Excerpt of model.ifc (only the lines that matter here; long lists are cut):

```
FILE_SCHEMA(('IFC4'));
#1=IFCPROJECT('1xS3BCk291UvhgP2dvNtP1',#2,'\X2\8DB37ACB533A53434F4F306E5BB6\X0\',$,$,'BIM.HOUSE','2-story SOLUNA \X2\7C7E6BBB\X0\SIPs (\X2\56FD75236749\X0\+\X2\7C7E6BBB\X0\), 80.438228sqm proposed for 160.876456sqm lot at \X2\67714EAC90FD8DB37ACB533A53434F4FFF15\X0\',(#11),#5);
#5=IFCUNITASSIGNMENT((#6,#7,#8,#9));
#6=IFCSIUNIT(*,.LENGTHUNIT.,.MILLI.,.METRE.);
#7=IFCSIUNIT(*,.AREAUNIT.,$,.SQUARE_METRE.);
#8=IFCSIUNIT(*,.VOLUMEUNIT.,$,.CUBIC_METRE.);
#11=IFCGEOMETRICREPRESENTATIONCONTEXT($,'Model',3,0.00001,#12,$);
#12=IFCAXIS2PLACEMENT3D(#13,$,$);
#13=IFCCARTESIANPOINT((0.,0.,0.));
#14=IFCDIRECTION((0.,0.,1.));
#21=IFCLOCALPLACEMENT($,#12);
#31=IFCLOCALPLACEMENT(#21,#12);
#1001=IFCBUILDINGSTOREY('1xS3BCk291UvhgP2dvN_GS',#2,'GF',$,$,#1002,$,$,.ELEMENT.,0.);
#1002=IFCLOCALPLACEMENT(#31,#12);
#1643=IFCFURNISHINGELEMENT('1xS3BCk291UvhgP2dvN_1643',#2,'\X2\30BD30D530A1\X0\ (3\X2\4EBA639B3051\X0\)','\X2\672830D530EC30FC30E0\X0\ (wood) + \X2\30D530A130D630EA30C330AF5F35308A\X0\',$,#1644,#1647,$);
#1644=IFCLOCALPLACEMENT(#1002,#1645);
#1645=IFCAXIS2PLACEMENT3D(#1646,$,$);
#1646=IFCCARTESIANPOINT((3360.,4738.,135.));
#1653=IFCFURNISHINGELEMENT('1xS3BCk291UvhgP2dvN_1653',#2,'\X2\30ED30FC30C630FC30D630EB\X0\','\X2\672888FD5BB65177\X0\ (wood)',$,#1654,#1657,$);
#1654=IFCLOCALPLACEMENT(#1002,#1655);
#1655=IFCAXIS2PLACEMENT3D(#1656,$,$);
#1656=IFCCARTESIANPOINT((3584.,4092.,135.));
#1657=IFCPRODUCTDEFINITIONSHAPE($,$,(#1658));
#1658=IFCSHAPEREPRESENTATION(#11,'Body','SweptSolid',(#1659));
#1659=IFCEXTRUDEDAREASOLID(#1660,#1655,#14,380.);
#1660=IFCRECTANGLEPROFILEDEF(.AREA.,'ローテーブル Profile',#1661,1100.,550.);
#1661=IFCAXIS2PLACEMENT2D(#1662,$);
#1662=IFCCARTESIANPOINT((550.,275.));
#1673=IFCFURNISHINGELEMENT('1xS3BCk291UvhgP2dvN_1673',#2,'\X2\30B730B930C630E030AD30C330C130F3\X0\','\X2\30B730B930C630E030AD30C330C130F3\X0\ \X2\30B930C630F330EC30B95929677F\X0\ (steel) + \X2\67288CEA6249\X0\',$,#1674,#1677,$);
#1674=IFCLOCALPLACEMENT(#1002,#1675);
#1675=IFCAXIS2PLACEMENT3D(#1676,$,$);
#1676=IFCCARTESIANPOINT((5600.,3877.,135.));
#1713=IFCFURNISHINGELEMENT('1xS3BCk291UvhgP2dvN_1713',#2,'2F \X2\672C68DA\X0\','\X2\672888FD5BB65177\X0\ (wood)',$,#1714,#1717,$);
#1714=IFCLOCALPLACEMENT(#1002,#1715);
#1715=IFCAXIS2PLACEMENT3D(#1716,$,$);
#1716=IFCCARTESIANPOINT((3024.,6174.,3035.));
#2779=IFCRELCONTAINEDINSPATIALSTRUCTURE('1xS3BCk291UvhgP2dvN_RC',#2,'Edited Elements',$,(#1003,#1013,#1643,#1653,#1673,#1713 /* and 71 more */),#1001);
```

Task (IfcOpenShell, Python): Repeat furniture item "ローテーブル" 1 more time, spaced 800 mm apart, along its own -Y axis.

```python
import ifcopenshell
import ifcopenshell.api.geometry
import ifcopenshell.api.root
import ifcopenshell.util.element
import ifcopenshell.util.placement
import ifcopenshell.util.unit

model = ifcopenshell.open("model.ifc")
unit_scale = ifcopenshell.util.unit.calculate_unit_scale(model)


def reuse_history(source, copy):
    """copy_class also copies each property set's owner history, people and application; keep the originals."""
    for rel in copy.IsDefinedBy:
        if rel.is_a("IfcRelDefinesByProperties") and (history := rel.RelatingPropertyDefinition.OwnerHistory):
            rel.RelatingPropertyDefinition.OwnerHistory = source.OwnerHistory
            ifcopenshell.util.element.remove_deep2(model, history)


source = model.by_guid("1xS3BCk291UvhgP2dvN_1653")
base = ifcopenshell.util.placement.get_local_placement(source.ObjectPlacement)
step = -base[:3, 1] * 0.8 / unit_scale

for i in range(1, 2):
    copy = ifcopenshell.api.root.copy_class(model, product=source)
    copy.Representation = ifcopenshell.util.element.copy_deep(
        model, source.Representation, exclude=["IfcGeometricRepresentationContext", "IfcRepresentationMap"]
    )
    reuse_history(source, copy)
    matrix = base.copy()
    matrix[:3, 3] += i * step
    print("added at", matrix[:3, 3].round(3) + 0.0)
    ifcopenshell.api.geometry.edit_object_placement(model, product=copy, matrix=matrix, is_si=False)

model.write("model_rev.ifc")
```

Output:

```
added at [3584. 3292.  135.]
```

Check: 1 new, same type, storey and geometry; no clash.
